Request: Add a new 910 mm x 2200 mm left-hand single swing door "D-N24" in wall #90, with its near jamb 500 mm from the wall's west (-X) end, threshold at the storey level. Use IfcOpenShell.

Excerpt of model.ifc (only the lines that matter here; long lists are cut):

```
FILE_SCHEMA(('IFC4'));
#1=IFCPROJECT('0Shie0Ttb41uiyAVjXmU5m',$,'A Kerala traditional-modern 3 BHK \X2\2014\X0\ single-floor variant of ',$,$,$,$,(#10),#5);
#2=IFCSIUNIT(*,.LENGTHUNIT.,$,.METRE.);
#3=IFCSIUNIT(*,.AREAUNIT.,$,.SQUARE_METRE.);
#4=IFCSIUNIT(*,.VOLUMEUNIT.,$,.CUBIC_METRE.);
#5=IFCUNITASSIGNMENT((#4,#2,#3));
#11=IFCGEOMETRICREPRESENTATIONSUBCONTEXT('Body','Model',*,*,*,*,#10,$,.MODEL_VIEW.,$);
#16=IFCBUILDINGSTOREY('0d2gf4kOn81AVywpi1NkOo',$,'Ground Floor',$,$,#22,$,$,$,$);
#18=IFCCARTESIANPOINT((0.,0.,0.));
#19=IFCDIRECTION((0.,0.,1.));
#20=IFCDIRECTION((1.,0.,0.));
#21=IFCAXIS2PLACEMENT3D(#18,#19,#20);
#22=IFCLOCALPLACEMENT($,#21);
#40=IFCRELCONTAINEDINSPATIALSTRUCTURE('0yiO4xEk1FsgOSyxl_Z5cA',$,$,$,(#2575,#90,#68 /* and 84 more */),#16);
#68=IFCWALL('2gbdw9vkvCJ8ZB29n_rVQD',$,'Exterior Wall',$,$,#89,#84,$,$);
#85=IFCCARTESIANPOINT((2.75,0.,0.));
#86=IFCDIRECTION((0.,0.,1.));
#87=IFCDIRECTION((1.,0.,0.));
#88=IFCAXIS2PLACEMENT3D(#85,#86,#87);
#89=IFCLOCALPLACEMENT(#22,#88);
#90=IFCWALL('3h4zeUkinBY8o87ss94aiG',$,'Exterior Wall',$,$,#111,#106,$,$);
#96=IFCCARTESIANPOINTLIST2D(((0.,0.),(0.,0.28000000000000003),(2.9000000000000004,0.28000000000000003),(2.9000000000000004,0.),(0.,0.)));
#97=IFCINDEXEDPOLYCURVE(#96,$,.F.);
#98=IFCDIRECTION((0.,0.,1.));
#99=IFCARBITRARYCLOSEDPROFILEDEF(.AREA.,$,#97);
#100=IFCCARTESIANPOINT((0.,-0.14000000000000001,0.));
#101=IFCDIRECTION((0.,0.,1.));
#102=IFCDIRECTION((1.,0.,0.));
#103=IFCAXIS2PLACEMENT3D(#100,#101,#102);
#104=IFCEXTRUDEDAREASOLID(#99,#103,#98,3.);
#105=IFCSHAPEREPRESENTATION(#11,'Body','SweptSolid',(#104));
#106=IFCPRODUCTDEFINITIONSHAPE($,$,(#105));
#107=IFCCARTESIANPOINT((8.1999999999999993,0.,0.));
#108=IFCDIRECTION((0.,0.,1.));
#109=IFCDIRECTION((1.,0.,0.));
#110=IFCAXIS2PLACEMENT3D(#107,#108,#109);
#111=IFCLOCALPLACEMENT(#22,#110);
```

```python
import numpy as np
import ifcopenshell
import ifcopenshell.api.feature
import ifcopenshell.api.geometry
import ifcopenshell.api.root
import ifcopenshell.api.spatial
import ifcopenshell.geom
import ifcopenshell.util.element
import ifcopenshell.util.placement
import ifcopenshell.util.representation
import ifcopenshell.util.shape
import ifcopenshell.util.unit

model = ifcopenshell.open("model.ifc")
unit_scale = ifcopenshell.util.unit.calculate_unit_scale(model)
settings = ifcopenshell.geom.settings()


def volume(element):
    """Net volume in cubic metres, openings subtracted."""
    shape = ifcopenshell.geom.create_shape(settings, element)
    return ifcopenshell.util.shape.get_volume(shape.geometry)


wall = model.by_id(90)
storey = ifcopenshell.util.element.get_container(wall, ifc_class="IfcBuildingStorey")
context = ifcopenshell.util.representation.get_context(model, "Model", "Body", "MODEL_VIEW")
before = volume(wall)

width, height, from_end, sill = 0.91, 2.2, 0.5, 0.0  # metres

# The wall runs along its own X axis, and the end named is its -X end.
wall_shape = ifcopenshell.geom.create_shape(settings, wall)
x, y, z = ifcopenshell.util.shape.get_vertices(wall_shape.geometry).T
start = x.min() + from_end
face, thickness = float(y.min()), float(y.max() - y.min())
wall_matrix = ifcopenshell.util.placement.get_local_placement(wall.ObjectPlacement)
level = ifcopenshell.util.placement.get_local_placement(storey.ObjectPlacement)[2, 3]


def in_wall(x, y):
    """Placement at x, y metres in the wall's axes, at sill height."""
    matrix = wall_matrix.copy()
    matrix[:, 3] = wall_matrix @ np.array([x / unit_scale, y / unit_scale, 0.0, 1.0])
    matrix[2, 3] = level + sill / unit_scale
    return matrix


# Opening: a box that overshoots both wall faces by 50 mm.
opening = ifcopenshell.api.root.create_entity(model, ifc_class="IfcOpeningElement", predefined_type="OPENING")
box = ifcopenshell.api.geometry.add_wall_representation(
    model, context=context, length=width, height=height, thickness=thickness + 0.1
)
ifcopenshell.api.geometry.assign_representation(model, product=opening, representation=box)
ifcopenshell.api.geometry.edit_object_placement(model, product=opening, matrix=in_wall(start, face - 0.05), is_si=False)
ifcopenshell.api.feature.add_feature(model, feature=opening, element=wall)

door = ifcopenshell.api.root.create_entity(model, ifc_class="IfcDoor", name="D-N24", predefined_type="DOOR")
door.OverallWidth, door.OverallHeight = width / unit_scale, height / unit_scale
door.OperationType = "SINGLE_SWING_LEFT"
body = ifcopenshell.api.geometry.add_door_representation(
    model,
    context=context,
    overall_width=door.OverallWidth,
    overall_height=door.OverallHeight,
    operation_type="SINGLE_SWING_LEFT",
    lining_properties={"LiningDepth": thickness / unit_scale, "ThresholdDepth": thickness / unit_scale},
)
ifcopenshell.api.geometry.assign_representation(model, product=door, representation=body)
ifcopenshell.api.spatial.assign_container(model, products=[door], relating_structure=storey)
ifcopenshell.api.feature.add_filling(model, opening=opening, element=door)

# The lining spans the wall, so the door starts at the wall face.
ifcopenshell.api.geometry.edit_object_placement(model, product=door, matrix=in_wall(start, face), is_si=False)

after = volume(wall)

print(f"wall volume {before:.3f} -> {after:.3f} m3")

model.write("model_rev.ifc")
```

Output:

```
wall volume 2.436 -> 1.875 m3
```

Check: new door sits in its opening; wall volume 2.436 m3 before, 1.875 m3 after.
